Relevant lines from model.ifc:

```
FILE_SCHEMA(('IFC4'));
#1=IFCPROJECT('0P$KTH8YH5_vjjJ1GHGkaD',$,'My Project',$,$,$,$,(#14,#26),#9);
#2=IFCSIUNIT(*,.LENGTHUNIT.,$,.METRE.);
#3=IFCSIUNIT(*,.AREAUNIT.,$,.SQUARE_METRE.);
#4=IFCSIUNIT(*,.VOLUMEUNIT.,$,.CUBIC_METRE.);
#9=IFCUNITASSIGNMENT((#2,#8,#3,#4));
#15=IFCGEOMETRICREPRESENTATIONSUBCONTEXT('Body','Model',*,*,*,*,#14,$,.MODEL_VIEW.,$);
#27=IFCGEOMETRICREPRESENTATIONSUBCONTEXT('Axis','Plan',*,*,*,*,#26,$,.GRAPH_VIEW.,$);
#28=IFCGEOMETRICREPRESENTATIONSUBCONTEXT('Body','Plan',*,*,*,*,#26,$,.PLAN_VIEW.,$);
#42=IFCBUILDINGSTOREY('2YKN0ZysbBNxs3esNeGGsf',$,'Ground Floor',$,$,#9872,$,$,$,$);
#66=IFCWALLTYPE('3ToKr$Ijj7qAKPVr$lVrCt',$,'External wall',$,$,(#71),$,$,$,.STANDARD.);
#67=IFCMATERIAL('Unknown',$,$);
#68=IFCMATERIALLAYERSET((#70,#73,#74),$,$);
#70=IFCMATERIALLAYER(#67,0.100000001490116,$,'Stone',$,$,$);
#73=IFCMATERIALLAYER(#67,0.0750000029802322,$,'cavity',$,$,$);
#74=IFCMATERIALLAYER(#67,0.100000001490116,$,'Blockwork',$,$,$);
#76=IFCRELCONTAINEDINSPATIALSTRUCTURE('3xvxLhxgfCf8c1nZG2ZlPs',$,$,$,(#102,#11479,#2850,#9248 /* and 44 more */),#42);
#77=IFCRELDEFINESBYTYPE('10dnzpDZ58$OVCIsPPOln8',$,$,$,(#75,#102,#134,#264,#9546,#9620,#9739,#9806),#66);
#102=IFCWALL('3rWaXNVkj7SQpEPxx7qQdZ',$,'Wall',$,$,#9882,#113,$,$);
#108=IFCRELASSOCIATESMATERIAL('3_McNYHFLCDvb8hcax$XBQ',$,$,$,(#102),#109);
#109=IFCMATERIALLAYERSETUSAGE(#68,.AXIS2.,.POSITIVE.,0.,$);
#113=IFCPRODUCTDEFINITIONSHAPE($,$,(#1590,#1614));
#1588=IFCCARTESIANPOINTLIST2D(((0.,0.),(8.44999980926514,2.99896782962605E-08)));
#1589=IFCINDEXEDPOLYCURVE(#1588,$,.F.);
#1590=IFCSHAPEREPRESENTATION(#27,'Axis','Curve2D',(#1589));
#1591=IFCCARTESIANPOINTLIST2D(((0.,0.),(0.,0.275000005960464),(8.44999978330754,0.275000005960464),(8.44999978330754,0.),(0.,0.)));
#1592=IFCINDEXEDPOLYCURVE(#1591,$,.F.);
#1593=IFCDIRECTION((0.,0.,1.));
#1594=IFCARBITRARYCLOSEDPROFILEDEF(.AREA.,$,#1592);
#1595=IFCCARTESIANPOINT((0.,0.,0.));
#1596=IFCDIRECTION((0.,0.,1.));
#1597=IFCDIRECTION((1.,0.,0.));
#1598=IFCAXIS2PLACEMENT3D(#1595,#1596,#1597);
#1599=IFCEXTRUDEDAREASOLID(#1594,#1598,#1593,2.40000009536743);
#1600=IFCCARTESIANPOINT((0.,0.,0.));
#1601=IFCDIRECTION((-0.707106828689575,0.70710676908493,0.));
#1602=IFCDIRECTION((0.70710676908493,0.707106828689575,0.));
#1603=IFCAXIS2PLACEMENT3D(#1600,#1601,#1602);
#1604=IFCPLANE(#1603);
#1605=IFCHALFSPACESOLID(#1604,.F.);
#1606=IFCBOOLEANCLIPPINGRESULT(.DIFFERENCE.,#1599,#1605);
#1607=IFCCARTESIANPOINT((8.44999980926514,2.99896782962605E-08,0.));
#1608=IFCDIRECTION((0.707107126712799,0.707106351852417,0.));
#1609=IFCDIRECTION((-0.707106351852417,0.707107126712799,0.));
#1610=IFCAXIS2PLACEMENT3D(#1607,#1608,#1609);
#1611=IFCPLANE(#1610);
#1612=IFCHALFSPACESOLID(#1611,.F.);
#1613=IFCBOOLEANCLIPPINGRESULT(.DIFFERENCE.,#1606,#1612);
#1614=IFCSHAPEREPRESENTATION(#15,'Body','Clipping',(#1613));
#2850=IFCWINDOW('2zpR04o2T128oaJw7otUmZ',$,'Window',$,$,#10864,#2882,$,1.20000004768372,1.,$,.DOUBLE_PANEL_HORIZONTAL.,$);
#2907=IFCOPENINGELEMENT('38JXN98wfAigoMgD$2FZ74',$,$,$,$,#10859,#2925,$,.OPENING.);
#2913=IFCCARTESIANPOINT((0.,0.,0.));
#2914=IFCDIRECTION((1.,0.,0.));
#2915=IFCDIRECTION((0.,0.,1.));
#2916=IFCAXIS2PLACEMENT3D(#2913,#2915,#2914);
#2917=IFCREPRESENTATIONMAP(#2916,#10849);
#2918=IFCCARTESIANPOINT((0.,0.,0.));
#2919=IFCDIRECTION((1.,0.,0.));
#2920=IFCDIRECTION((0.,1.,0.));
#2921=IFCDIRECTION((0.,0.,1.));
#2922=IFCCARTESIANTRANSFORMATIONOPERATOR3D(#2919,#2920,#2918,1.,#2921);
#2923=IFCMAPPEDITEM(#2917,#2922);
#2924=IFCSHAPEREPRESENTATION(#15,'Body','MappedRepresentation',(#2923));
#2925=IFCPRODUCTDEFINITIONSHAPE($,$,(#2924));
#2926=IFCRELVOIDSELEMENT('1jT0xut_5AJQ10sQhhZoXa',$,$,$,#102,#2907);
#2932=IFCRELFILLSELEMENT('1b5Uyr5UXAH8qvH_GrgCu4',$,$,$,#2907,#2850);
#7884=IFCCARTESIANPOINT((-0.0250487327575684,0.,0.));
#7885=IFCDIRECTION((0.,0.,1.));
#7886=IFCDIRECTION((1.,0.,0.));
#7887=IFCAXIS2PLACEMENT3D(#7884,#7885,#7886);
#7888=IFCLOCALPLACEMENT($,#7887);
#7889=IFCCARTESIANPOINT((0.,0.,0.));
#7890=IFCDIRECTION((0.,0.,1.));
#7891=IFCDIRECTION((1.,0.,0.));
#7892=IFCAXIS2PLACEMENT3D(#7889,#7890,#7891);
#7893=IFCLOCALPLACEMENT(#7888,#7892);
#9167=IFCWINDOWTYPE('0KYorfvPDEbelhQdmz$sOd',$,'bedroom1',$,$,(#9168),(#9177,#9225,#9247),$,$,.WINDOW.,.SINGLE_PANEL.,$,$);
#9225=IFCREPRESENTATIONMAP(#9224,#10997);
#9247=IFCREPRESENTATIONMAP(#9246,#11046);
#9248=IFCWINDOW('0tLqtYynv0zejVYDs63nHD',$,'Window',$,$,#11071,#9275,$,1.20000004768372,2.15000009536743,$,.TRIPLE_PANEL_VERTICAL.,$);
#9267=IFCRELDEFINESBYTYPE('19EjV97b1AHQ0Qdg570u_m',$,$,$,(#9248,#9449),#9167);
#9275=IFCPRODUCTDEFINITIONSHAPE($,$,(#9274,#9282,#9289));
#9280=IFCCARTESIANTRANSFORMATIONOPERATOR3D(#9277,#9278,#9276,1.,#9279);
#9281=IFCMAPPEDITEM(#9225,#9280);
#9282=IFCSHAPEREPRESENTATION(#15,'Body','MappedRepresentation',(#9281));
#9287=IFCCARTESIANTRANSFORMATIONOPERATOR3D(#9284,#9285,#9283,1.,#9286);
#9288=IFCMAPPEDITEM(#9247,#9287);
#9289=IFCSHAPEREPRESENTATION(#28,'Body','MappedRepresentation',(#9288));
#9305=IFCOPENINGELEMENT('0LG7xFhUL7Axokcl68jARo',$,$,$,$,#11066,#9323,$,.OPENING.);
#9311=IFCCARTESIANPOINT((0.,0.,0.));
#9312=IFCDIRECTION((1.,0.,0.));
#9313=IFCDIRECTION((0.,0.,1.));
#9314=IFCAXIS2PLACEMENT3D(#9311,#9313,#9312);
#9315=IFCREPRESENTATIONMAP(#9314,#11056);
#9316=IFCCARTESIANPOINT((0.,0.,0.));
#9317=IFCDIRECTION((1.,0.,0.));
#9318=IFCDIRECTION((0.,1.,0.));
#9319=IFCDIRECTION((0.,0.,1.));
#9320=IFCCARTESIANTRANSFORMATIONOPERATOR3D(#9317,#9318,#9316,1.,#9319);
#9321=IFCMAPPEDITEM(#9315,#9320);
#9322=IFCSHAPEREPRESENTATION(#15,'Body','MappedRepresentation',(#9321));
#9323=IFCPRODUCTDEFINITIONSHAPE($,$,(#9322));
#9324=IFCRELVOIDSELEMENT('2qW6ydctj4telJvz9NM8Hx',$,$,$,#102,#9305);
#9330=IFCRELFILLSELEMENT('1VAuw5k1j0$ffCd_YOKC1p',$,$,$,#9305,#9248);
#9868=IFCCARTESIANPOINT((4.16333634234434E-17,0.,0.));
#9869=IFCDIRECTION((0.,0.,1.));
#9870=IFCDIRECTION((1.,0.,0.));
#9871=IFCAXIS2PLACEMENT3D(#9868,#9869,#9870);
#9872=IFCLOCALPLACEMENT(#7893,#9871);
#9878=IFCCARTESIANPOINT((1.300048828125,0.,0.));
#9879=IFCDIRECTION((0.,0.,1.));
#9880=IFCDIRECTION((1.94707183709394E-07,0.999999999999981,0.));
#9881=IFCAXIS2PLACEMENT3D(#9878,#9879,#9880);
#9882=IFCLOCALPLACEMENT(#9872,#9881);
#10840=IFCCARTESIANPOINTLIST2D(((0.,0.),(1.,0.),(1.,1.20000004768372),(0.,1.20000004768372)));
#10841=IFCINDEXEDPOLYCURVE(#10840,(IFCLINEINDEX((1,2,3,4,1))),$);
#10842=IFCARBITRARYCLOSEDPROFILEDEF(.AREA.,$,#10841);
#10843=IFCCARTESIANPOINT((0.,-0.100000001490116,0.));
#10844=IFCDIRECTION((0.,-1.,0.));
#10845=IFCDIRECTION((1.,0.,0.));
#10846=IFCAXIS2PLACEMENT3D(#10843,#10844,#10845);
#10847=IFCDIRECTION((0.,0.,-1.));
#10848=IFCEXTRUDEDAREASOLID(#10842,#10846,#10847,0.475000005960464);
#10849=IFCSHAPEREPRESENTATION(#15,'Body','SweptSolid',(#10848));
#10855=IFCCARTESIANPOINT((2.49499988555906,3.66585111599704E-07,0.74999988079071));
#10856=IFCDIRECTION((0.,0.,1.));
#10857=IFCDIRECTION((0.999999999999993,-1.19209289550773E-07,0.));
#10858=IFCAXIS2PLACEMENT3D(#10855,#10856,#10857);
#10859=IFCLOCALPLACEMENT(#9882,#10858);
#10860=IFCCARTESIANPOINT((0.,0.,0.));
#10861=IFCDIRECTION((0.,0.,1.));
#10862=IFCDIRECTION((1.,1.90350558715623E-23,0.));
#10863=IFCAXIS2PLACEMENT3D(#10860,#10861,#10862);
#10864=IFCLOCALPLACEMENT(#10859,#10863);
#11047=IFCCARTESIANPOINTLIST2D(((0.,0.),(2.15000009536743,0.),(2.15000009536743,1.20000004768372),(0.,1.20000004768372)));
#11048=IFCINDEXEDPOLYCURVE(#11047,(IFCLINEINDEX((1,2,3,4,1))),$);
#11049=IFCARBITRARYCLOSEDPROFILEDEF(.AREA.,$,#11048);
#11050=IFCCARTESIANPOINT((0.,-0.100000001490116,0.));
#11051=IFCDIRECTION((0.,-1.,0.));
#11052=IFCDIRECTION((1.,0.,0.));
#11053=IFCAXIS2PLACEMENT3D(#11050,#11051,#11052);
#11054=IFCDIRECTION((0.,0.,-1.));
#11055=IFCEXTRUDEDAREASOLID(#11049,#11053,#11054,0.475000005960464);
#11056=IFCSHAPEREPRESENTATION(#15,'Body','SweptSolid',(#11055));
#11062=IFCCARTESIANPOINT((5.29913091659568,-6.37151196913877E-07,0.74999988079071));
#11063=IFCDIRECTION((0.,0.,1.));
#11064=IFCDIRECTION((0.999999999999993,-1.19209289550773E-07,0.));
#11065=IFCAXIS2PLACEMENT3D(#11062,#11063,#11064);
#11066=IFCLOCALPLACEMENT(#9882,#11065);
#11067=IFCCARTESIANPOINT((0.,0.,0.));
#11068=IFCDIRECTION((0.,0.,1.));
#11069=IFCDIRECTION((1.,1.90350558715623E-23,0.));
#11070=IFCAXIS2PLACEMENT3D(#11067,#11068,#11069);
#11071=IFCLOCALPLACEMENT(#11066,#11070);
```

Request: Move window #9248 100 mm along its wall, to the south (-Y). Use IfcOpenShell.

```python
import ifcopenshell
import ifcopenshell.api.geometry
import ifcopenshell.util.placement
import ifcopenshell.util.unit

model = ifcopenshell.open("model.ifc")
unit_scale = ifcopenshell.util.unit.calculate_unit_scale(model)

window = model.by_guid("0tLqtYynv0zejVYDs63nHD")
opening = window.FillsVoids[0].RelatingOpeningElement
wall = opening.VoidsElements[0].RelatingBuildingElement

wall_matrix = ifcopenshell.util.placement.get_local_placement(wall.ObjectPlacement)
shift = wall_matrix[:3, 0] * -0.1 / unit_scale
before = ifcopenshell.util.placement.get_local_placement(window.ObjectPlacement)[:3, 3].copy()

# The window is placed relative to its opening, so it follows when the opening moves.
matrix = ifcopenshell.util.placement.get_local_placement(opening.ObjectPlacement)
matrix[:3, 3] += shift
ifcopenshell.api.geometry.edit_object_placement(
    model, product=opening, matrix=matrix, is_si=False, should_transform_children=True
)

after = ifcopenshell.util.placement.get_local_placement(window.ObjectPlacement)[:3, 3]
print("window moved by", (after - before).round(3) + 0.0)

model.write("model-out.ifc")
```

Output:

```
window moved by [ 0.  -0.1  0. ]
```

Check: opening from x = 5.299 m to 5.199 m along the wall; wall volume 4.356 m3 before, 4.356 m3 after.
